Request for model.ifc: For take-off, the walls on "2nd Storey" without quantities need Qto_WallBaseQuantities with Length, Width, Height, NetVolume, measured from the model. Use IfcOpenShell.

First a look at what the model holds.

```python
import ifcopenshell
import ifcopenshell.util.element
import ifcopenshell.util.unit

model = ifcopenshell.open("model.ifc")
print(model.schema)
for unit_type in ("LENGTHUNIT", "AREAUNIT", "VOLUMEUNIT"):
    print(unit_type, ifcopenshell.util.unit.calculate_unit_scale(model, unit_type))
storey = next(s for s in model.by_type("IfcBuildingStorey") if s.Name == "2nd Storey")
walls = [e for e in ifcopenshell.util.element.get_decomposition(storey) if e.is_a("IfcWall")]
for e in sorted(walls, key=lambda e: e.id()):
    print(e.id(), e.is_a(), e.Name, list(ifcopenshell.util.element.get_psets(e, qtos_only=True)), sep=" | ")
```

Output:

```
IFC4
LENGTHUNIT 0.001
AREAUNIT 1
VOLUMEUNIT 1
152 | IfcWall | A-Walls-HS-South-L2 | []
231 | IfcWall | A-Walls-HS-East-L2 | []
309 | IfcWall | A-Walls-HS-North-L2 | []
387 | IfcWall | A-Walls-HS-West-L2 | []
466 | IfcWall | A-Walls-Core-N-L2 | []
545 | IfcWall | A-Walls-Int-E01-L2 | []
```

```python
import ifcopenshell
import ifcopenshell.api.pset
import ifcopenshell.geom
import ifcopenshell.util.element
import ifcopenshell.util.shape
import ifcopenshell.util.unit

model = ifcopenshell.open("model.ifc")
unit_scale = ifcopenshell.util.unit.calculate_unit_scale(model)
volume_scale = ifcopenshell.util.unit.calculate_unit_scale(model, "VOLUMEUNIT")
settings = ifcopenshell.geom.settings()

storey = next(s for s in model.by_type("IfcBuildingStorey") if s.Name == "2nd Storey")
walls = [e for e in ifcopenshell.util.element.get_decomposition(storey) if e.is_a("IfcWall")]

for e in sorted(walls, key=lambda e: e.id()):
    if ifcopenshell.util.element.get_psets(e, qtos_only=True, should_inherit=False):
        continue
    # Geometry comes back in metres, in the element's own axes.
    shape = ifcopenshell.geom.create_shape(settings, e)
    values = {
        "Length": ifcopenshell.util.shape.get_x(shape.geometry) / unit_scale,
        "Width": ifcopenshell.util.shape.get_y(shape.geometry) / unit_scale,
        "Height": ifcopenshell.util.shape.get_z(shape.geometry) / unit_scale,
        "NetVolume": ifcopenshell.util.shape.get_volume(shape.geometry) / volume_scale,
    }
    qto = ifcopenshell.api.pset.add_qto(model, product=e, name="Qto_WallBaseQuantities")
    ifcopenshell.api.pset.edit_qto(model, qto=qto, properties=values)
    print(e.id(), {k: round(v, 3) for k, v in values.items()})

model.write("model_rev.ifc")
```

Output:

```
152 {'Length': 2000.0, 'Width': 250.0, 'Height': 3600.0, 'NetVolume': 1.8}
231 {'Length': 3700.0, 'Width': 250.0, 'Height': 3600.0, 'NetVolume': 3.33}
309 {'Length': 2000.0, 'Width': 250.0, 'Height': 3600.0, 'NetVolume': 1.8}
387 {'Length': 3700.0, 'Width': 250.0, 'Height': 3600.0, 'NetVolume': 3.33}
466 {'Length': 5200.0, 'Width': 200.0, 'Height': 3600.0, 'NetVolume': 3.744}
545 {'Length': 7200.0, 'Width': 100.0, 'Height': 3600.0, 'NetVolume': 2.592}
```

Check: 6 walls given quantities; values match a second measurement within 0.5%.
